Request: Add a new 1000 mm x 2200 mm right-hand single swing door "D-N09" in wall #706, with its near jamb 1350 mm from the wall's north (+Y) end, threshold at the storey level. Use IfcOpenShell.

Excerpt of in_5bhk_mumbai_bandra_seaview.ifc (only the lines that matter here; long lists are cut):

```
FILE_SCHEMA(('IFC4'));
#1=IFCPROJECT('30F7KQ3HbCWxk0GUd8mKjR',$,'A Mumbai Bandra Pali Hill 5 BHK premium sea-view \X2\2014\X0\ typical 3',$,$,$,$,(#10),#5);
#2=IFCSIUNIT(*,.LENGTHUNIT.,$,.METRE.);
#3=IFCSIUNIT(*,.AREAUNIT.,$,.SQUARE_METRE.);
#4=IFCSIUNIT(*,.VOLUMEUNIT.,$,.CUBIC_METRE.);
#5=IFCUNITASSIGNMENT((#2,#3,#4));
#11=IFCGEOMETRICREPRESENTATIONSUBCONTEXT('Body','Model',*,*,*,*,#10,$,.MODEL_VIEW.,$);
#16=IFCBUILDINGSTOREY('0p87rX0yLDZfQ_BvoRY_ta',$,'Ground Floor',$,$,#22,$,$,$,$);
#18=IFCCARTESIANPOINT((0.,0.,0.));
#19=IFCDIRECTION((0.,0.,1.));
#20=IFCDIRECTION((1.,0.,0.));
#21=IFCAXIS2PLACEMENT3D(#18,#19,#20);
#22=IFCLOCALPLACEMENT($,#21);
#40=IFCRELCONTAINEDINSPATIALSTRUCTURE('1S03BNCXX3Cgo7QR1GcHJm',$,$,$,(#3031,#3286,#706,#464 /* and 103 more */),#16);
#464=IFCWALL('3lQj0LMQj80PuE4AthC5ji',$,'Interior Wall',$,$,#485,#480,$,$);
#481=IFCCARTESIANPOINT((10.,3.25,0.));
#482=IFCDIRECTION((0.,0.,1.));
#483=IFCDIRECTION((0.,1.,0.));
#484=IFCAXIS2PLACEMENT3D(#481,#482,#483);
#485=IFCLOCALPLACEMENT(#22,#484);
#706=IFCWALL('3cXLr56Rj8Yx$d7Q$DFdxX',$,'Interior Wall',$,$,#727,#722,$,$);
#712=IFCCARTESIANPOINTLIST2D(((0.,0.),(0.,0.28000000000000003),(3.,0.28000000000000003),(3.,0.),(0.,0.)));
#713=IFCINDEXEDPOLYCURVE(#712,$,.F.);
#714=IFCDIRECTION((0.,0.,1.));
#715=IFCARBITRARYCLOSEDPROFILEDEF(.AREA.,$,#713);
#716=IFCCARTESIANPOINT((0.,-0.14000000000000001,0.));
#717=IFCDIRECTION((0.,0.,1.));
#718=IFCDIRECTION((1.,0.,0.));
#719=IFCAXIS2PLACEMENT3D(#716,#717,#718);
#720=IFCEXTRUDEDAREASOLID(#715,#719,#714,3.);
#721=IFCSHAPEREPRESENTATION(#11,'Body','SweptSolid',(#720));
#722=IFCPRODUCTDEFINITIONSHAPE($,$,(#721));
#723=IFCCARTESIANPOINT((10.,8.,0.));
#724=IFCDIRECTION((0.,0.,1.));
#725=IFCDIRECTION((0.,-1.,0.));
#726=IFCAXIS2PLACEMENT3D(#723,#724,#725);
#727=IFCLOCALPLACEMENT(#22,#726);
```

```python
import numpy as np
import ifcopenshell
import ifcopenshell.api.feature
import ifcopenshell.api.geometry
import ifcopenshell.api.root
import ifcopenshell.api.spatial
import ifcopenshell.geom
import ifcopenshell.util.element
import ifcopenshell.util.placement
import ifcopenshell.util.representation
import ifcopenshell.util.shape
import ifcopenshell.util.unit

model = ifcopenshell.open("in_5bhk_mumbai_bandra_seaview.ifc")
unit_scale = ifcopenshell.util.unit.calculate_unit_scale(model)
settings = ifcopenshell.geom.settings()


def volume(element):
    """Net volume in cubic metres, openings subtracted."""
    shape = ifcopenshell.geom.create_shape(settings, element)
    return ifcopenshell.util.shape.get_volume(shape.geometry)


wall = model.by_guid("3cXLr56Rj8Yx$d7Q$DFdxX")
storey = ifcopenshell.util.element.get_container(wall, ifc_class="IfcBuildingStorey")
context = ifcopenshell.util.representation.get_context(model, "Model", "Body", "MODEL_VIEW")
before = volume(wall)

width, height, from_end, sill = 1, 2.2, 1.35, 0.0  # metres

# The wall runs along its own X axis, and the end named is its -X end.
wall_shape = ifcopenshell.geom.create_shape(settings, wall)
x, y, z = ifcopenshell.util.shape.get_vertices(wall_shape.geometry).T
start = x.min() + from_end
face, thickness = float(y.min()), float(y.max() - y.min())
wall_matrix = ifcopenshell.util.placement.get_local_placement(wall.ObjectPlacement)
level = ifcopenshell.util.placement.get_local_placement(storey.ObjectPlacement)[2, 3]


def in_wall(x, y):
    """Placement at x, y metres in the wall's axes, at sill height."""
    matrix = wall_matrix.copy()
    matrix[:, 3] = wall_matrix @ np.array([x / unit_scale, y / unit_scale, 0.0, 1.0])
    matrix[2, 3] = level + sill / unit_scale
    return matrix


# Opening: a box that overshoots both wall faces by 50 mm.
opening = ifcopenshell.api.root.create_entity(model, ifc_class="IfcOpeningElement", predefined_type="OPENING")
box = ifcopenshell.api.geometry.add_wall_representation(
    model, context=context, length=width, height=height, thickness=thickness + 0.1
)
ifcopenshell.api.geometry.assign_representation(model, product=opening, representation=box)
ifcopenshell.api.geometry.edit_object_placement(model, product=opening, matrix=in_wall(start, face - 0.05), is_si=False)
ifcopenshell.api.feature.add_feature(model, feature=opening, element=wall)

door = ifcopenshell.api.root.create_entity(model, ifc_class="IfcDoor", name="D-N09", predefined_type="DOOR")
door.OverallWidth, door.OverallHeight = width / unit_scale, height / unit_scale
door.OperationType = "SINGLE_SWING_RIGHT"
body = ifcopenshell.api.geometry.add_door_representation(
    model,
    context=context,
    overall_width=door.OverallWidth,
    overall_height=door.OverallHeight,
    operation_type="SINGLE_SWING_RIGHT",
    lining_properties={"LiningDepth": thickness / unit_scale, "ThresholdDepth": thickness / unit_scale},
)
ifcopenshell.api.geometry.assign_representation(model, product=door, representation=body)
ifcopenshell.api.spatial.assign_container(model, products=[door], relating_structure=storey)
ifcopenshell.api.feature.add_filling(model, opening=opening, element=door)

# The lining spans the wall, so the door starts at the wall face.
ifcopenshell.api.geometry.edit_object_placement(model, product=door, matrix=in_wall(start, face), is_si=False)

after = volume(wall)

print(f"wall volume {before:.3f} -> {after:.3f} m3")

model.write("in_5bhk_mumbai_bandra_seaview_v2.ifc")
```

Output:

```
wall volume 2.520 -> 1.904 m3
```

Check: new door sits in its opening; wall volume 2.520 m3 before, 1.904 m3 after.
